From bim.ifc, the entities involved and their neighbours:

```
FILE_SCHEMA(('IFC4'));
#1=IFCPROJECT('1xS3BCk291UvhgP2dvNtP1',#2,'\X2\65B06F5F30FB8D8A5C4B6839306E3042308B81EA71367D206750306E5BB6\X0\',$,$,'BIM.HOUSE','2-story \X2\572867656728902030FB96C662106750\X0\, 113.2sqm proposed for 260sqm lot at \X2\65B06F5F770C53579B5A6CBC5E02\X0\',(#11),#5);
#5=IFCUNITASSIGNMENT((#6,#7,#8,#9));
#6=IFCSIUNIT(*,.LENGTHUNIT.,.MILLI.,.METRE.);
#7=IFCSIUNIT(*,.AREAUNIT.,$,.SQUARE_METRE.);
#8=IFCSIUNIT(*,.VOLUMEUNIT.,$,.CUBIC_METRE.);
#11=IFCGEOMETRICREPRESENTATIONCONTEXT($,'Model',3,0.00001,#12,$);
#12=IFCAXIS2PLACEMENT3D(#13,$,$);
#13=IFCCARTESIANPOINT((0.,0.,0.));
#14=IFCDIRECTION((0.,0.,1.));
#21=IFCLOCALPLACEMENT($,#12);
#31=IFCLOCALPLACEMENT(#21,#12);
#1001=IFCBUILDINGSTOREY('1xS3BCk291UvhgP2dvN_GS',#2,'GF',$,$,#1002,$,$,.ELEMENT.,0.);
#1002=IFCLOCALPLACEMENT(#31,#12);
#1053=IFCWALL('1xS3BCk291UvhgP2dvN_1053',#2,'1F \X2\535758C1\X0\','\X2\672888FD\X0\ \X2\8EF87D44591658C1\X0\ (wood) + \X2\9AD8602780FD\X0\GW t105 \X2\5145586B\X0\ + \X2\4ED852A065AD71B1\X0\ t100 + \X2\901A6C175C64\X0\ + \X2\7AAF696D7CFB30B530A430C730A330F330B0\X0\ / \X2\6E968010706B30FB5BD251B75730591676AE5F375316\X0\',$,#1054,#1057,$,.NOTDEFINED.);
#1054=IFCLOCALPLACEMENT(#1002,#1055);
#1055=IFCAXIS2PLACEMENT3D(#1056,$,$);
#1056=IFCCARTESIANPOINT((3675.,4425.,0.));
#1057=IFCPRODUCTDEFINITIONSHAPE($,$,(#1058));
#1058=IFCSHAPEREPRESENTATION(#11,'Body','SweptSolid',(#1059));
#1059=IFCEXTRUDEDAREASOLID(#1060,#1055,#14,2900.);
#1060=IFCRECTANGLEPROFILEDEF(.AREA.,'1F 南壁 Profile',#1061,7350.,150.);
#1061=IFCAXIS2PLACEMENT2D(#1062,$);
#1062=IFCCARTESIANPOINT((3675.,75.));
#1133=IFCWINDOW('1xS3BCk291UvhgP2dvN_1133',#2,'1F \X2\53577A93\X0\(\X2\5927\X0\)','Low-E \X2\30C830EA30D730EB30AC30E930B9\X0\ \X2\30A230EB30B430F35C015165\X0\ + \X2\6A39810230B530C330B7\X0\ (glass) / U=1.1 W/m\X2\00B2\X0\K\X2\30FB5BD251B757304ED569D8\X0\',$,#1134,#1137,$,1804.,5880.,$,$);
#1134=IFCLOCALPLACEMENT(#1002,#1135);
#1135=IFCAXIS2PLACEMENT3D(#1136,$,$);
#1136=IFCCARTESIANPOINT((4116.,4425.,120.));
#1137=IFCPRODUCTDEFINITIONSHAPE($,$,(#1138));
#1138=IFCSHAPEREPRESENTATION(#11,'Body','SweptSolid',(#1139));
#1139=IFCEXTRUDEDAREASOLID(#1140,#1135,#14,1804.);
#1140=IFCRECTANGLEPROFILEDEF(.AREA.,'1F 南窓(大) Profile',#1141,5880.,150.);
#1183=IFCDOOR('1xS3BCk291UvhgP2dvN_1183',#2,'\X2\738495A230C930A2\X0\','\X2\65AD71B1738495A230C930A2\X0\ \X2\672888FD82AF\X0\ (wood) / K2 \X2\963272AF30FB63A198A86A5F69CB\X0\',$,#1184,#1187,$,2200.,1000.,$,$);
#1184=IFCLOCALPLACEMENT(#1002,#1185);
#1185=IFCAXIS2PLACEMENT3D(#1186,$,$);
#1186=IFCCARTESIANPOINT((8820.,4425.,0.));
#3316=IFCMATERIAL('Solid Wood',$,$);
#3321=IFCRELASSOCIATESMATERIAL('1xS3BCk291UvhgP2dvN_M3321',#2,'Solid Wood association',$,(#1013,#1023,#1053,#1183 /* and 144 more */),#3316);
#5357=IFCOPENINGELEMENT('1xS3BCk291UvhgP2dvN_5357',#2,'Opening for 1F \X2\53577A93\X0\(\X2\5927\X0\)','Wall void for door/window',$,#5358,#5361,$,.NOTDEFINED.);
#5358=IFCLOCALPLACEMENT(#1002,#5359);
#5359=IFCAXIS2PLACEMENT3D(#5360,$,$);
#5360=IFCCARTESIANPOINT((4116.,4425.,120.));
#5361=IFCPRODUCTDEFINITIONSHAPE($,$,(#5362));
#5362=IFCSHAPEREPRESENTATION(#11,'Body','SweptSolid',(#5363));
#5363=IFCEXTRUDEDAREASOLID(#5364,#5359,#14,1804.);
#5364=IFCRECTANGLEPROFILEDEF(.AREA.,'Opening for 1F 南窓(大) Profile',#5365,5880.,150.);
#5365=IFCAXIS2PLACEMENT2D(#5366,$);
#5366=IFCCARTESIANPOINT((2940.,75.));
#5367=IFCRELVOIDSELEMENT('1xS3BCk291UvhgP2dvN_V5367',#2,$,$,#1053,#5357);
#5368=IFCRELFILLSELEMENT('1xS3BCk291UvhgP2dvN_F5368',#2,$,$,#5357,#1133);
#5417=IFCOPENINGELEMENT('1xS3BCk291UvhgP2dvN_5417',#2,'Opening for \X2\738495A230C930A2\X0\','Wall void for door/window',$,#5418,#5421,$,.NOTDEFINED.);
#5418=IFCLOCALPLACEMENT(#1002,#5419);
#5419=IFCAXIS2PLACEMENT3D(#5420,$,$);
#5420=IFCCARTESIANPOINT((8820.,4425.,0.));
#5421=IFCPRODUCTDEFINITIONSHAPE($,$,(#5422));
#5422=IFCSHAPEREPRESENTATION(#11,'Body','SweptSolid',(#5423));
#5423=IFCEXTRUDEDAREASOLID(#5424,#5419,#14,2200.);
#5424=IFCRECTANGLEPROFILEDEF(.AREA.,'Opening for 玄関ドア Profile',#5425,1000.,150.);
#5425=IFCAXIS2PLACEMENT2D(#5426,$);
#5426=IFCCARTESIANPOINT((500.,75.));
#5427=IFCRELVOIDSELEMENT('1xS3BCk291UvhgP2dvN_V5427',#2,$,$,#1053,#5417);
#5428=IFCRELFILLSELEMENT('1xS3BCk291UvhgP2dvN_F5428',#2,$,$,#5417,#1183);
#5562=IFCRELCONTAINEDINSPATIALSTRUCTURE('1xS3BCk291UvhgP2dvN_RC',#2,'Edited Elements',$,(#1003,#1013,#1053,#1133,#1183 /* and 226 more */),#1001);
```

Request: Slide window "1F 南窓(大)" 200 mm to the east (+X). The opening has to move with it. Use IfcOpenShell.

```python
import ifcopenshell
import ifcopenshell.api.geometry
import ifcopenshell.util.placement
import ifcopenshell.util.unit

model = ifcopenshell.open("bim.ifc")
unit_scale = ifcopenshell.util.unit.calculate_unit_scale(model)

window = model.by_id(1133)
opening = window.FillsVoids[0].RelatingOpeningElement
wall = opening.VoidsElements[0].RelatingBuildingElement

wall_matrix = ifcopenshell.util.placement.get_local_placement(wall.ObjectPlacement)
shift = wall_matrix[:3, 0] * 0.2 / unit_scale
before = ifcopenshell.util.placement.get_local_placement(window.ObjectPlacement)[:3, 3].copy()

# The window is not placed relative to its opening, so move both.
for product in (opening, window):
    matrix = ifcopenshell.util.placement.get_local_placement(product.ObjectPlacement)
    matrix[:3, 3] += shift
    ifcopenshell.api.geometry.edit_object_placement(model, product=product, matrix=matrix, is_si=False)

after = ifcopenshell.util.placement.get_local_placement(window.ObjectPlacement)[:3, 3]
print("window moved by", (after - before).round(3) + 0.0)

model.write("bim_updated.ifc")
```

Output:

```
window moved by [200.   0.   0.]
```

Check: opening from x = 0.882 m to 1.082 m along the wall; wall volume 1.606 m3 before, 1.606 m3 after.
